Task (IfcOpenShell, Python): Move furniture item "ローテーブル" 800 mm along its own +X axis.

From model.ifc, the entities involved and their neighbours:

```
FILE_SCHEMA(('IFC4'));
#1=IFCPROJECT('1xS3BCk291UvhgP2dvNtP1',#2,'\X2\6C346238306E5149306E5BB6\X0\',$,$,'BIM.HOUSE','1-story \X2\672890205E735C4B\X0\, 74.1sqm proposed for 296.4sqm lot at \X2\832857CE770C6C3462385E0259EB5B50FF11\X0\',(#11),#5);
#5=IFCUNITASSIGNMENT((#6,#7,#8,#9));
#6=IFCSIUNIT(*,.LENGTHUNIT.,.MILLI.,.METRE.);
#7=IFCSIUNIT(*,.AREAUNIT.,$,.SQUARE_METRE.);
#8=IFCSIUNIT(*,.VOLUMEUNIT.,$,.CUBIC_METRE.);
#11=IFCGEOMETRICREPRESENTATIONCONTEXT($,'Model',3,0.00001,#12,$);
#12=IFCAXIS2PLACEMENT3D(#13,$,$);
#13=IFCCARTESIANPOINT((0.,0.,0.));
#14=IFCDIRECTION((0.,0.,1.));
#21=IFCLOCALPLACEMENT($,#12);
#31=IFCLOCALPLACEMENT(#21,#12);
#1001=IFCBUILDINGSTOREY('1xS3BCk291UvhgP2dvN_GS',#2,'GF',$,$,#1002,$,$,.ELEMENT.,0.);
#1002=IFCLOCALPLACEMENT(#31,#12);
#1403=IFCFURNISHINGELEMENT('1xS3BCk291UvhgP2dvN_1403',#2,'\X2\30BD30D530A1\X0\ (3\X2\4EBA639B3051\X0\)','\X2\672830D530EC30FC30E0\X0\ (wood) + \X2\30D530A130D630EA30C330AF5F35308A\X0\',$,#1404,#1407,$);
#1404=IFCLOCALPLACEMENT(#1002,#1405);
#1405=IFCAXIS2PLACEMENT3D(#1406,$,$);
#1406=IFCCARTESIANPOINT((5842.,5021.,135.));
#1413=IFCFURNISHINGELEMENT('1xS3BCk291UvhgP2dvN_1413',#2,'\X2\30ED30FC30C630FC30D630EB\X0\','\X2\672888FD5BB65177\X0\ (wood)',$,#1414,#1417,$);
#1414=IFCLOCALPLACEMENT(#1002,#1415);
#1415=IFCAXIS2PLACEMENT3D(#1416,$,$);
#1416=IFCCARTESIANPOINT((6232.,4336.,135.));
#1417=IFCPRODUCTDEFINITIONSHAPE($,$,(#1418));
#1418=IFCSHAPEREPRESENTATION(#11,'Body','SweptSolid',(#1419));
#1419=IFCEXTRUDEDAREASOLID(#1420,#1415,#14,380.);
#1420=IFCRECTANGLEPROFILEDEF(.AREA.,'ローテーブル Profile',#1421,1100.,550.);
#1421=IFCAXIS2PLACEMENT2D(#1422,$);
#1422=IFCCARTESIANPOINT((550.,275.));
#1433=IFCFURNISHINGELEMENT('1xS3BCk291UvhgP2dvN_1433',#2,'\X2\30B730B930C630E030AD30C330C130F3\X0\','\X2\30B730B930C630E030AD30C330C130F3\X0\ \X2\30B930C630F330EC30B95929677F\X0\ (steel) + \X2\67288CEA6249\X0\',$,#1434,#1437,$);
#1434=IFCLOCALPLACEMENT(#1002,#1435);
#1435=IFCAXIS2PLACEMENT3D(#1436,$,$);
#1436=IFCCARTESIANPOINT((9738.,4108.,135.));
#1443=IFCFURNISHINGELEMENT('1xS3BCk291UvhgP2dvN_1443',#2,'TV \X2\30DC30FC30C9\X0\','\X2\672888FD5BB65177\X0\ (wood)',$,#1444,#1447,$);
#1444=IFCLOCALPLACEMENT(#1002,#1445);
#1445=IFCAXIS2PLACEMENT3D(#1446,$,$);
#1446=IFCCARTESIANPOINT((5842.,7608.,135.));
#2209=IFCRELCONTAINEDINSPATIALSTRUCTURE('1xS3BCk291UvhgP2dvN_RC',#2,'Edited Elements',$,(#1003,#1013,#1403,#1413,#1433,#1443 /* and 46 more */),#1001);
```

```python
import ifcopenshell
import ifcopenshell.api.geometry
import ifcopenshell.util.placement
import ifcopenshell.util.unit

model = ifcopenshell.open("model.ifc")
unit_scale = ifcopenshell.util.unit.calculate_unit_scale(model)

item = model.by_id(1413)
matrix = ifcopenshell.util.placement.get_local_placement(item.ObjectPlacement)
matrix[:3, 3] += matrix[:3, 0] * 0.8 / unit_scale
ifcopenshell.api.geometry.edit_object_placement(model, product=item, matrix=matrix, is_si=False)

print(ifcopenshell.util.placement.get_local_placement(item.ObjectPlacement).round(3) + 0.0)

model.write("model_updated.ifc")
```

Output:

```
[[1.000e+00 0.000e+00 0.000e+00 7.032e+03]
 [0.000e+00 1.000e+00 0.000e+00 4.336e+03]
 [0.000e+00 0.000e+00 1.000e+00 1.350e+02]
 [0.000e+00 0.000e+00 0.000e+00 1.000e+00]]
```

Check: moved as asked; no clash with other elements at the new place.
